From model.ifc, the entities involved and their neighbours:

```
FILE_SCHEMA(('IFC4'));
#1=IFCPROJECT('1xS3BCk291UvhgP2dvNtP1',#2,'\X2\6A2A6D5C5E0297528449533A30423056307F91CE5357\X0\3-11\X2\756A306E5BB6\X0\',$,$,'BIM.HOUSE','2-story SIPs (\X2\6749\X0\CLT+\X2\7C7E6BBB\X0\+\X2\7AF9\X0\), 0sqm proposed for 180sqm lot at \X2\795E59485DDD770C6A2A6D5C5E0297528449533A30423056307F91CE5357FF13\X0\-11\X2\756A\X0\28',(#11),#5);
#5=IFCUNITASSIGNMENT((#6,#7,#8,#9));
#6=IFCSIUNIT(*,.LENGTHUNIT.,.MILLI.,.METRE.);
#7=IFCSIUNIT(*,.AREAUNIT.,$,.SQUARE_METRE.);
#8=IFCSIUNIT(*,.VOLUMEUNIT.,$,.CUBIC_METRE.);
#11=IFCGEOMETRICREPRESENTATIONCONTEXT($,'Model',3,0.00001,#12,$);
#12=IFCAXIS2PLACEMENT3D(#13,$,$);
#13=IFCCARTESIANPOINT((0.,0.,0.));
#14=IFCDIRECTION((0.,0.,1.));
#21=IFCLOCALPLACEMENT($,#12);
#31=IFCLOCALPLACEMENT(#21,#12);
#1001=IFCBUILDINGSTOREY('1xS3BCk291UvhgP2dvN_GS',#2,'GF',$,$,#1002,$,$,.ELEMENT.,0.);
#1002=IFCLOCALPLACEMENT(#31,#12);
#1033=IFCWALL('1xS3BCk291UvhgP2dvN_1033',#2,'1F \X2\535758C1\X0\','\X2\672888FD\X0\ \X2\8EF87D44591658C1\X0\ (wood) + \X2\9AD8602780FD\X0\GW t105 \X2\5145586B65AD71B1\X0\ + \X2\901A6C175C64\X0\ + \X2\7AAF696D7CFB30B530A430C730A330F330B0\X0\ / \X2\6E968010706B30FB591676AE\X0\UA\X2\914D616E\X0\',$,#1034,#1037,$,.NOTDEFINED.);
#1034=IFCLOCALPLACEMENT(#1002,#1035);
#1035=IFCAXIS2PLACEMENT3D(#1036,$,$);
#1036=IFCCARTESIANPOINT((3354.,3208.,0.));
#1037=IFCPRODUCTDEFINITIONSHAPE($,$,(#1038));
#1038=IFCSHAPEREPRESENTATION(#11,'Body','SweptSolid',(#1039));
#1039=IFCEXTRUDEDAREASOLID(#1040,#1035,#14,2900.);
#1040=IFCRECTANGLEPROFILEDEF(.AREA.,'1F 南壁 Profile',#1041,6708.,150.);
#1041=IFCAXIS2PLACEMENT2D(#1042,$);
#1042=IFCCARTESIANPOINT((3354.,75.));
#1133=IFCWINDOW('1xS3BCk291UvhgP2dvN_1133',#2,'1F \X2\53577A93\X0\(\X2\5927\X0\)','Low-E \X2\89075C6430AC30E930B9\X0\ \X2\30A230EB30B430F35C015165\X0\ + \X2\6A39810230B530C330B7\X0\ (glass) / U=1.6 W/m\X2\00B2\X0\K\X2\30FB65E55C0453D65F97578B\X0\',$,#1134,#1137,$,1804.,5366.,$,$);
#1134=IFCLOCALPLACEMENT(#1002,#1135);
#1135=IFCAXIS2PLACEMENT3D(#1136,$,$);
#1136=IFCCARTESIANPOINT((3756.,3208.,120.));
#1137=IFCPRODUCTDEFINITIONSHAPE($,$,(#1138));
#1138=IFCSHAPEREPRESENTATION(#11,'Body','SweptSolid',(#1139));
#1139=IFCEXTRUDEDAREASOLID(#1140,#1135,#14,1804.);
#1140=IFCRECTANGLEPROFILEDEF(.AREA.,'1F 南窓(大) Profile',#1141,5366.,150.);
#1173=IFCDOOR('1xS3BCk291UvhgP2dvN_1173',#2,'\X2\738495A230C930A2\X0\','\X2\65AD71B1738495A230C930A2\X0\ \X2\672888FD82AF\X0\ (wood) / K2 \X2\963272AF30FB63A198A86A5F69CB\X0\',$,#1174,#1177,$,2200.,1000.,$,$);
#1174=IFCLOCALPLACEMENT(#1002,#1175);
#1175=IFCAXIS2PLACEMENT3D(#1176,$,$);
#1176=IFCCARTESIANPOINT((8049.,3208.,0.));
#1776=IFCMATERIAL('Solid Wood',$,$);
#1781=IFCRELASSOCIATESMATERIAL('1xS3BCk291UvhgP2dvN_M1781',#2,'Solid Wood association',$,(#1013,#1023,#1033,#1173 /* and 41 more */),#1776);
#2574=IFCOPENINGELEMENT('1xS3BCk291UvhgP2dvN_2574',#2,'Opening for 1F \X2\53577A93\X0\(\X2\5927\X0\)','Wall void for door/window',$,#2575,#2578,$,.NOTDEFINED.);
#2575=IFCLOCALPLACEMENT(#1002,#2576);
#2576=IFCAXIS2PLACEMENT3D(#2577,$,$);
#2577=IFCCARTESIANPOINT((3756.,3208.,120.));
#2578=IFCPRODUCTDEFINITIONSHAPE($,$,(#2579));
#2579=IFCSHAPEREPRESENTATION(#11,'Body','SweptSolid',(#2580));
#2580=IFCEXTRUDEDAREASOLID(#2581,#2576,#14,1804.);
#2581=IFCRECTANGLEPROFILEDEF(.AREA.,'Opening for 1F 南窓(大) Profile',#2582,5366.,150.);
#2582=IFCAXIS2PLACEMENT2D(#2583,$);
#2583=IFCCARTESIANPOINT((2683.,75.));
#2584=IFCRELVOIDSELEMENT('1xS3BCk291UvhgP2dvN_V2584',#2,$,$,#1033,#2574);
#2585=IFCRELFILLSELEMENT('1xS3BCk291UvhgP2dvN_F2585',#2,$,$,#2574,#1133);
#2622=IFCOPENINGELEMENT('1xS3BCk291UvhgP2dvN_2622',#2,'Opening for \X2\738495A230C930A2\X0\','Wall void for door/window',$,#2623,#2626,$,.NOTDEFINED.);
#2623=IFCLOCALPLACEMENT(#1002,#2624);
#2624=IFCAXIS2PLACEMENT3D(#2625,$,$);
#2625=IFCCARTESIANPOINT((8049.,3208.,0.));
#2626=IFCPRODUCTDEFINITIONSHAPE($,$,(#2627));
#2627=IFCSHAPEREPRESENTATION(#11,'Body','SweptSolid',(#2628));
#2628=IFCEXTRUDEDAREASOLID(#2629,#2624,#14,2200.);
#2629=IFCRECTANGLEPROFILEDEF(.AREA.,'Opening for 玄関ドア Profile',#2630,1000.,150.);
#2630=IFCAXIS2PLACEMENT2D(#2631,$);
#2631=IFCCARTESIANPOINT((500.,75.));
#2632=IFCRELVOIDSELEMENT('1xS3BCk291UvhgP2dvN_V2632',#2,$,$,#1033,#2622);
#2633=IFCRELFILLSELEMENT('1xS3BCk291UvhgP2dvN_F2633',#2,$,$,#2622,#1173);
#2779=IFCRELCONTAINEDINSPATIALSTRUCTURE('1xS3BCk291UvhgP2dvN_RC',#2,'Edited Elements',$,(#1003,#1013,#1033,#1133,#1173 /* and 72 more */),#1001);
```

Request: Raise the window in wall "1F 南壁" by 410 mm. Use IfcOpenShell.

```python
import numpy as np
import ifcopenshell
import ifcopenshell.api.geometry
import ifcopenshell.util.placement
import ifcopenshell.util.unit

model = ifcopenshell.open("model.ifc")
unit_scale = ifcopenshell.util.unit.calculate_unit_scale(model)

window = model.by_guid("1xS3BCk291UvhgP2dvN_1133")
opening = window.FillsVoids[0].RelatingOpeningElement
dz = 410.0

shift = np.array([0.0, 0.0, dz])
# The window is not placed relative to its opening, so move both.
for product in (opening, window):
    matrix = ifcopenshell.util.placement.get_local_placement(product.ObjectPlacement)
    matrix[:3, 3] += shift
    ifcopenshell.api.geometry.edit_object_placement(model, product=product, matrix=matrix, is_si=False)

print(f"moved by {dz * unit_scale:+.3f} m")

model.write("model-out.ifc")
```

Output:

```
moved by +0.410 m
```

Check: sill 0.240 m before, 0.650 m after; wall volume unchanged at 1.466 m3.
